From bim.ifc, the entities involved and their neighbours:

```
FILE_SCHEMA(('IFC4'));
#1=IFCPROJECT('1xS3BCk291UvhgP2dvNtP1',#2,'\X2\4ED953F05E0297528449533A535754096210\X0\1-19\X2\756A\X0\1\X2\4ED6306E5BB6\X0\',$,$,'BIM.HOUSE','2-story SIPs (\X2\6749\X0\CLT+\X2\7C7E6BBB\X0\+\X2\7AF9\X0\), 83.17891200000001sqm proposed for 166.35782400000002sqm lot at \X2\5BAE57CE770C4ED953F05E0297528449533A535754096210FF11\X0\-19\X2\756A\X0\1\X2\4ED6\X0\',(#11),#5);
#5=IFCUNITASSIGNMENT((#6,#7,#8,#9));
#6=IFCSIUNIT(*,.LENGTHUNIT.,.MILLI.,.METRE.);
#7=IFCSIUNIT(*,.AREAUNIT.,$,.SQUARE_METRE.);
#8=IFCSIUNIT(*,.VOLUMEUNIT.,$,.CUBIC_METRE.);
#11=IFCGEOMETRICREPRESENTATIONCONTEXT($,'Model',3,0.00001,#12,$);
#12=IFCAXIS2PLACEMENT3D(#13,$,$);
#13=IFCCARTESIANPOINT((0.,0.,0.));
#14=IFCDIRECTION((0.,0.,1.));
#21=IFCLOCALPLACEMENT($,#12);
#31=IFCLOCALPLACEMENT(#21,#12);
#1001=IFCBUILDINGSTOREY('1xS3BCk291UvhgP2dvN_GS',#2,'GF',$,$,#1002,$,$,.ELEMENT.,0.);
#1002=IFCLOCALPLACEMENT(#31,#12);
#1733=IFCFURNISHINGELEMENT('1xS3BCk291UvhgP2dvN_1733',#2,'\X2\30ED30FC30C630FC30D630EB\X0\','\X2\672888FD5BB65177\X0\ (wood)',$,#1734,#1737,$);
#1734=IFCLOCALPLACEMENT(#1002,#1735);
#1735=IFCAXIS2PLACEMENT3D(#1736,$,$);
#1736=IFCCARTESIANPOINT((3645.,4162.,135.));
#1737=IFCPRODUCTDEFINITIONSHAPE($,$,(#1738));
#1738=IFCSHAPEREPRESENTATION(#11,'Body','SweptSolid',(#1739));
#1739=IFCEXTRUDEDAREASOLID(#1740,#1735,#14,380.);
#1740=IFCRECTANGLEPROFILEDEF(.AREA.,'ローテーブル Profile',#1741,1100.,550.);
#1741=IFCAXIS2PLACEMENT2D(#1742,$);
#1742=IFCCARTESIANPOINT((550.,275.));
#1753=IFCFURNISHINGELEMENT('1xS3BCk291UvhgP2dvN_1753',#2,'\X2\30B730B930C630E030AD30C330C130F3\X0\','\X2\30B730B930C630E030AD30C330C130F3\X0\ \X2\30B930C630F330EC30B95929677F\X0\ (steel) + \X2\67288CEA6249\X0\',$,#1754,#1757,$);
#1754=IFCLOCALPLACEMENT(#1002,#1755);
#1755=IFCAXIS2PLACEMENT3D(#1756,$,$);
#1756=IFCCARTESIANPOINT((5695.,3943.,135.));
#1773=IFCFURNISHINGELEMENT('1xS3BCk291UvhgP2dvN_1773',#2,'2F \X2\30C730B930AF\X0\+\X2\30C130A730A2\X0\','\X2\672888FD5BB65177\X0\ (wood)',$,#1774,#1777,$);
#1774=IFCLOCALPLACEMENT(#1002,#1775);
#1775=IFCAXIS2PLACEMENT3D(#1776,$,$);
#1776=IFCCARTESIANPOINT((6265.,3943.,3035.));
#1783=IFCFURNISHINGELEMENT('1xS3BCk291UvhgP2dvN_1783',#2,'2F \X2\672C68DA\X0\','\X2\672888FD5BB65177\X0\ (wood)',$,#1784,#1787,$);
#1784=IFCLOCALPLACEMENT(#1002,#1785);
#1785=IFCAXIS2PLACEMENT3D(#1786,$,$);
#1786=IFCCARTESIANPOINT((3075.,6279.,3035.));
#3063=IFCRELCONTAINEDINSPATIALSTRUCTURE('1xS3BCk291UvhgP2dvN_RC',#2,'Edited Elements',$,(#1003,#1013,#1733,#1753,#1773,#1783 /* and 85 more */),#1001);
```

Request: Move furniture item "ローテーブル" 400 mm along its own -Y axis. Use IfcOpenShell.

```python
import ifcopenshell
import ifcopenshell.api.geometry
import ifcopenshell.util.placement

model = ifcopenshell.open("bim.ifc")

item = model.by_guid("1xS3BCk291UvhgP2dvN_1733")
matrix = ifcopenshell.util.placement.get_local_placement(item.ObjectPlacement)
matrix[:3, 3] -= matrix[:3, 1] * 400.0
ifcopenshell.api.geometry.edit_object_placement(model, product=item, matrix=matrix, is_si=False)

print(ifcopenshell.util.placement.get_local_placement(item.ObjectPlacement).round(3) + 0.0)

model.write("bim_updated.ifc")
```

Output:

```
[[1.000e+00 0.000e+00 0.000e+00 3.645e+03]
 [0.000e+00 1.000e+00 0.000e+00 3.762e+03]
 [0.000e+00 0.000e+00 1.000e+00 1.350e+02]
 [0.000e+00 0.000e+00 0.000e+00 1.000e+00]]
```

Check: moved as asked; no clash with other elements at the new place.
